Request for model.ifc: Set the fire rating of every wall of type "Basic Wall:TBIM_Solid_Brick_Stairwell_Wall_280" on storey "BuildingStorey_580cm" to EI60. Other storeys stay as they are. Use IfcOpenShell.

First a look at what the model holds.

```python
import ifcopenshell
import ifcopenshell.util.element

model = ifcopenshell.open("model.ifc")
print(model.schema)
storey = next(s for s in model.by_type("IfcBuildingStorey") if s.Name == "BuildingStorey_580cm")
walls = [e for e in ifcopenshell.util.element.get_decomposition(storey) if e.is_a("IfcWall")]
seen = {}
for e in walls:
    element_type = ifcopenshell.util.element.get_type(e)
    key = (element_type.Name if element_type != e and element_type else None, ifcopenshell.util.element.get_pset(e, "Pset_WallCommon", "FireRating"))
    seen[key] = seen.get(key, 0) + 1
for (name, value), count in sorted(seen.items(), key=str):
    print(count, "x", name, "|", value)
```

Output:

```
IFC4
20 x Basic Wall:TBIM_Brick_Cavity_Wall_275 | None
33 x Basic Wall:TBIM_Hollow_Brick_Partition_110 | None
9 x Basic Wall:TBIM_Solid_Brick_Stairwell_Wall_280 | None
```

```python
import ifcopenshell
import ifcopenshell.api.pset
import ifcopenshell.util.element

model = ifcopenshell.open("model.ifc")

storey = next(s for s in model.by_type("IfcBuildingStorey") if s.Name == "BuildingStorey_580cm")
walls = [e for e in ifcopenshell.util.element.get_decomposition(storey) if e.is_a("IfcWall")]

count = 0
for e in walls:
    element_type = ifcopenshell.util.element.get_type(e)
    if element_type in (None, e) or element_type.Name != "Basic Wall:TBIM_Solid_Brick_Stairwell_Wall_280":
        continue
    # add_pset returns the element's existing set when there is one.
    pset = ifcopenshell.api.pset.add_pset(model, product=e, name="Pset_WallCommon")
    ifcopenshell.api.pset.edit_pset(model, pset=pset, properties={"FireRating": "EI60"})
    count += 1

print(count, "walls updated")

model.write("model_edited.ifc")
```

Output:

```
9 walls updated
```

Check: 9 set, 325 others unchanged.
